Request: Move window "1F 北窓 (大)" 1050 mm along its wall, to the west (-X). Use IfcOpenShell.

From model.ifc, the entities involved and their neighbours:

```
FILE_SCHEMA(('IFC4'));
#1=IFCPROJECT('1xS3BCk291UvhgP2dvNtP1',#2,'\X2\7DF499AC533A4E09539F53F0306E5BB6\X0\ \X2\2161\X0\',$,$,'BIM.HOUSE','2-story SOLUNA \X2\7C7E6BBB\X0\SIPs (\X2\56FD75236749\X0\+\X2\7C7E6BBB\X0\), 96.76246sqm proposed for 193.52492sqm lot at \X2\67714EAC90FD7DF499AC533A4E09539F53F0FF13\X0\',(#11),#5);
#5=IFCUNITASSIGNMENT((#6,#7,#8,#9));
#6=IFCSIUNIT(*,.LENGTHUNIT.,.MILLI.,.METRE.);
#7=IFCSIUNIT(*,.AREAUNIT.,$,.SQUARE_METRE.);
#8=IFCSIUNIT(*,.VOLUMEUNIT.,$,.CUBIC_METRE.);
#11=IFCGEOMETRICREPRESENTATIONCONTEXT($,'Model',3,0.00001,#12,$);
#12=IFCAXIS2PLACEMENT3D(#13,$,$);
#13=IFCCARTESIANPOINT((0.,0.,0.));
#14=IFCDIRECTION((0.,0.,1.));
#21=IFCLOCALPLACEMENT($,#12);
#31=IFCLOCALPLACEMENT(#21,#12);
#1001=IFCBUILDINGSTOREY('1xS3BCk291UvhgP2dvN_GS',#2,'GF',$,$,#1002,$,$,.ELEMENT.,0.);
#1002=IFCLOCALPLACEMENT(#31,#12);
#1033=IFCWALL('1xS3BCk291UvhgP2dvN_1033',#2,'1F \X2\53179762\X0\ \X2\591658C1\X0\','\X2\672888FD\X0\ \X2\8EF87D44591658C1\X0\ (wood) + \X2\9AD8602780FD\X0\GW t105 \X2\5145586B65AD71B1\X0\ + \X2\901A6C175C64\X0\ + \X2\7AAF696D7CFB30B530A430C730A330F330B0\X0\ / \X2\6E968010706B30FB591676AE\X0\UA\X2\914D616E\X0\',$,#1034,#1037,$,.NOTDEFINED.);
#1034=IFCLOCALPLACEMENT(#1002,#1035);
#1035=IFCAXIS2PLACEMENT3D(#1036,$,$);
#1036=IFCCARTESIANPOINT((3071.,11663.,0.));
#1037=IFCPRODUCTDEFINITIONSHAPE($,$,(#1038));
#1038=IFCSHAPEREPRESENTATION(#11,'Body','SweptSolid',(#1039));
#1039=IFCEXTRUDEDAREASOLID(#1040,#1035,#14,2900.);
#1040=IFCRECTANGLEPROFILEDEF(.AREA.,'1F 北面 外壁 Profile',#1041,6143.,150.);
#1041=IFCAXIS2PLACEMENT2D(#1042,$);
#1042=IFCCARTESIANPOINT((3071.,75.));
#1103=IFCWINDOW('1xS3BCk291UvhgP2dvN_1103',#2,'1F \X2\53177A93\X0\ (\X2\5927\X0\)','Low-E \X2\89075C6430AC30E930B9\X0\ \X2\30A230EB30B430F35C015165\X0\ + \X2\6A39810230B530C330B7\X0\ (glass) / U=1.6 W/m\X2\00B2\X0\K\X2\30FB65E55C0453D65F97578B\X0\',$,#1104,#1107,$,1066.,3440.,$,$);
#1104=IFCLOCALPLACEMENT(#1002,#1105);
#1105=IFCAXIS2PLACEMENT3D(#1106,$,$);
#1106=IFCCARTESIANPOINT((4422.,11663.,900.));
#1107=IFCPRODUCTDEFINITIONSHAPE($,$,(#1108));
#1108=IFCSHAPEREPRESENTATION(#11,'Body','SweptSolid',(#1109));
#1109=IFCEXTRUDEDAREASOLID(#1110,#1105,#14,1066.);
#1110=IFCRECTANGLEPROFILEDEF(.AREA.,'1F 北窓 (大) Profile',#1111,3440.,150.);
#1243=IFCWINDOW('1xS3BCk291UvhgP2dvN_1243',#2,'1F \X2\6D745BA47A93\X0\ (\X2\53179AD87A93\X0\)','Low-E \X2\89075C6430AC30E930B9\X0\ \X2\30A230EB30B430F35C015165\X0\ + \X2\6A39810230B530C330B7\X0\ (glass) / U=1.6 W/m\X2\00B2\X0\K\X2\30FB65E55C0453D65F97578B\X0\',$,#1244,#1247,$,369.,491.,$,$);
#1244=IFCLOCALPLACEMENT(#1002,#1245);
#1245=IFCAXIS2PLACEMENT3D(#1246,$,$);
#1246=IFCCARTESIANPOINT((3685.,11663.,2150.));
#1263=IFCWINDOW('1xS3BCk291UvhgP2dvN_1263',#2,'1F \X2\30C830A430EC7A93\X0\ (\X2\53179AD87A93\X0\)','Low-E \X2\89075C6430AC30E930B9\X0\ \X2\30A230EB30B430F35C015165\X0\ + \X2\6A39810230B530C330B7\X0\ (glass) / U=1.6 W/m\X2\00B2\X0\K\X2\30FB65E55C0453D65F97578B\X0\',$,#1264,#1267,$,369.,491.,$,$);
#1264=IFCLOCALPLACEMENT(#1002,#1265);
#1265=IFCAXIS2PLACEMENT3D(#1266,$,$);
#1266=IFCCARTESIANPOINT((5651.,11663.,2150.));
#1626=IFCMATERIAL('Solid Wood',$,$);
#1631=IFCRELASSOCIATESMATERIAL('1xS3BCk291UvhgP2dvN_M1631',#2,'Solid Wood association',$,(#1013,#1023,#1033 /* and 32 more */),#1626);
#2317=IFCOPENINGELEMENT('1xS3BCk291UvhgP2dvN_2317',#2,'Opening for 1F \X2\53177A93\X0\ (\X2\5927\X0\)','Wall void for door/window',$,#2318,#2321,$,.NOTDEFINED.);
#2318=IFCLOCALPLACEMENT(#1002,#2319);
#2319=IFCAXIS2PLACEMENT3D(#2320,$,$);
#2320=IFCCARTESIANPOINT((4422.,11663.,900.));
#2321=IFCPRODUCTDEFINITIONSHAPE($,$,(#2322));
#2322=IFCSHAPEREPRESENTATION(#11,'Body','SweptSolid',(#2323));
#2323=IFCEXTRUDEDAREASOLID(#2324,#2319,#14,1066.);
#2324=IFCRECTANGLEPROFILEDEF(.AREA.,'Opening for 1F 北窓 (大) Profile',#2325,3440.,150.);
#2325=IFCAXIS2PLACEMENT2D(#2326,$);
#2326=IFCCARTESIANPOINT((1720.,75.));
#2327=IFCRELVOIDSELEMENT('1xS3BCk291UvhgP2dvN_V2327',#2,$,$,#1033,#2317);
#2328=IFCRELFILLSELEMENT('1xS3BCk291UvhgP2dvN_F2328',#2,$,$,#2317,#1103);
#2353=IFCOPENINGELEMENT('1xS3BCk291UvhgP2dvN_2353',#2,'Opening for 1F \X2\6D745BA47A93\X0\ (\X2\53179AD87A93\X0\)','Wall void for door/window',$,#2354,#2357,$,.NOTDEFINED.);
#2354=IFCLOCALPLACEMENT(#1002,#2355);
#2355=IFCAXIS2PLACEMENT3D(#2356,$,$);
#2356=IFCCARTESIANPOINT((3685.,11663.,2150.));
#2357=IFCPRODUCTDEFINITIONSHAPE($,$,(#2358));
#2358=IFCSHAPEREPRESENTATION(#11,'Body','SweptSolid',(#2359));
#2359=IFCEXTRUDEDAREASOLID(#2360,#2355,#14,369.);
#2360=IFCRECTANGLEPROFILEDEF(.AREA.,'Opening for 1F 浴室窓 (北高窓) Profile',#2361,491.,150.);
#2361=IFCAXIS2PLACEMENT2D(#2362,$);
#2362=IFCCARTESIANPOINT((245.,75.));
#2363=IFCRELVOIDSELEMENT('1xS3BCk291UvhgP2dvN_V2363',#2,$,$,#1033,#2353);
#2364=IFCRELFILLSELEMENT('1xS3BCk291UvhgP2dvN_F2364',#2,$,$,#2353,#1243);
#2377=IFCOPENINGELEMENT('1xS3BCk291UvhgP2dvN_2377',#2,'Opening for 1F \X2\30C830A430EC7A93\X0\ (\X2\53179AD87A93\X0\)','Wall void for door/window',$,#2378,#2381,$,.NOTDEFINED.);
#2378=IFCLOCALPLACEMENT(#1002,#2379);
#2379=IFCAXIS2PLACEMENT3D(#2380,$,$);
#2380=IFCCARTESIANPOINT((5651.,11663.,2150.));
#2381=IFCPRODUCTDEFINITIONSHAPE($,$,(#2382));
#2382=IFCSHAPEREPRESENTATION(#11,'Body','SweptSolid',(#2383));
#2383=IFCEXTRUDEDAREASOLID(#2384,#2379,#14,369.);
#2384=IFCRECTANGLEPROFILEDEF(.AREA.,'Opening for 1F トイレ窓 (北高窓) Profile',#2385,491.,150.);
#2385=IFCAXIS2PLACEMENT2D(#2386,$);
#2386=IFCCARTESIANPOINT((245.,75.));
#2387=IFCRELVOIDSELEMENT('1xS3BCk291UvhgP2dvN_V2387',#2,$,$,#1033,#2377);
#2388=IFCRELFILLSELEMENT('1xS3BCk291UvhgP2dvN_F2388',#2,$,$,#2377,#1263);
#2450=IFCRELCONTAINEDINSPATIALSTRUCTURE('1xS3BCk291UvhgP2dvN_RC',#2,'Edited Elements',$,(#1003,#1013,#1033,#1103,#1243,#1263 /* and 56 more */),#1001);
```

```python
import ifcopenshell
import ifcopenshell.api.geometry
import ifcopenshell.util.placement
import ifcopenshell.util.unit

model = ifcopenshell.open("model.ifc")
unit_scale = ifcopenshell.util.unit.calculate_unit_scale(model)

window = model.by_id(1103)
opening = window.FillsVoids[0].RelatingOpeningElement
wall = opening.VoidsElements[0].RelatingBuildingElement

wall_matrix = ifcopenshell.util.placement.get_local_placement(wall.ObjectPlacement)
shift = wall_matrix[:3, 0] * -1.05 / unit_scale
before = ifcopenshell.util.placement.get_local_placement(window.ObjectPlacement)[:3, 3].copy()

# The window is not placed relative to its opening, so move both.
for product in (opening, window):
    matrix = ifcopenshell.util.placement.get_local_placement(product.ObjectPlacement)
    matrix[:3, 3] += shift
    ifcopenshell.api.geometry.edit_object_placement(model, product=product, matrix=matrix, is_si=False)

after = ifcopenshell.util.placement.get_local_placement(window.ObjectPlacement)[:3, 3]
print("window moved by", (after - before).round(3) + 0.0)

model.write("model_v2.ifc")
```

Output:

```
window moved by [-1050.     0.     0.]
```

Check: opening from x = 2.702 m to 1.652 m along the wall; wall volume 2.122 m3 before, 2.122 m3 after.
